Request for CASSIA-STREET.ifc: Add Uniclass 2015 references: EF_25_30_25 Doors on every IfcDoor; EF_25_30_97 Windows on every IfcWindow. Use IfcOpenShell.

First a look at what the model holds.

```python
import ifcopenshell

model = ifcopenshell.open("CASSIA-STREET.ifc")
print(model.schema)
print("classifications:", [c.Name for c in model.by_type("IfcClassification")])
for ifc_class in ("IfcDoor", "IfcRoof", "IfcStair", "IfcWall", "IfcWindow"):
    print(ifc_class, len(model.by_type(ifc_class)))
```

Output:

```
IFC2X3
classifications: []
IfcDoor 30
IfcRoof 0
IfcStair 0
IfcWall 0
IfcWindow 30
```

```python
import ifcopenshell
import ifcopenshell.api.classification

model = ifcopenshell.open("CASSIA-STREET.ifc")

# IFC2X3 requires Source and Edition and has no link from the project to the system.
system = model.create_entity("IfcClassification", Source="NBS", Edition="2015", Name="Uniclass 2015")

codes = {
    "IfcDoor": ("EF_25_30_25", "Doors"),
    "IfcWindow": ("EF_25_30_97", "Windows"),
}
for ifc_class, (code, name) in codes.items():
    products = model.by_type(ifc_class)
    ifcopenshell.api.classification.add_reference(
        model, products=products, classification=system, identification=code, name=name
    )
    print(code, len(products))

model.write("CASSIA-STREET_v2.ifc")
```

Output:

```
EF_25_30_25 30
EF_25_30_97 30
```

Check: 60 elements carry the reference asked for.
